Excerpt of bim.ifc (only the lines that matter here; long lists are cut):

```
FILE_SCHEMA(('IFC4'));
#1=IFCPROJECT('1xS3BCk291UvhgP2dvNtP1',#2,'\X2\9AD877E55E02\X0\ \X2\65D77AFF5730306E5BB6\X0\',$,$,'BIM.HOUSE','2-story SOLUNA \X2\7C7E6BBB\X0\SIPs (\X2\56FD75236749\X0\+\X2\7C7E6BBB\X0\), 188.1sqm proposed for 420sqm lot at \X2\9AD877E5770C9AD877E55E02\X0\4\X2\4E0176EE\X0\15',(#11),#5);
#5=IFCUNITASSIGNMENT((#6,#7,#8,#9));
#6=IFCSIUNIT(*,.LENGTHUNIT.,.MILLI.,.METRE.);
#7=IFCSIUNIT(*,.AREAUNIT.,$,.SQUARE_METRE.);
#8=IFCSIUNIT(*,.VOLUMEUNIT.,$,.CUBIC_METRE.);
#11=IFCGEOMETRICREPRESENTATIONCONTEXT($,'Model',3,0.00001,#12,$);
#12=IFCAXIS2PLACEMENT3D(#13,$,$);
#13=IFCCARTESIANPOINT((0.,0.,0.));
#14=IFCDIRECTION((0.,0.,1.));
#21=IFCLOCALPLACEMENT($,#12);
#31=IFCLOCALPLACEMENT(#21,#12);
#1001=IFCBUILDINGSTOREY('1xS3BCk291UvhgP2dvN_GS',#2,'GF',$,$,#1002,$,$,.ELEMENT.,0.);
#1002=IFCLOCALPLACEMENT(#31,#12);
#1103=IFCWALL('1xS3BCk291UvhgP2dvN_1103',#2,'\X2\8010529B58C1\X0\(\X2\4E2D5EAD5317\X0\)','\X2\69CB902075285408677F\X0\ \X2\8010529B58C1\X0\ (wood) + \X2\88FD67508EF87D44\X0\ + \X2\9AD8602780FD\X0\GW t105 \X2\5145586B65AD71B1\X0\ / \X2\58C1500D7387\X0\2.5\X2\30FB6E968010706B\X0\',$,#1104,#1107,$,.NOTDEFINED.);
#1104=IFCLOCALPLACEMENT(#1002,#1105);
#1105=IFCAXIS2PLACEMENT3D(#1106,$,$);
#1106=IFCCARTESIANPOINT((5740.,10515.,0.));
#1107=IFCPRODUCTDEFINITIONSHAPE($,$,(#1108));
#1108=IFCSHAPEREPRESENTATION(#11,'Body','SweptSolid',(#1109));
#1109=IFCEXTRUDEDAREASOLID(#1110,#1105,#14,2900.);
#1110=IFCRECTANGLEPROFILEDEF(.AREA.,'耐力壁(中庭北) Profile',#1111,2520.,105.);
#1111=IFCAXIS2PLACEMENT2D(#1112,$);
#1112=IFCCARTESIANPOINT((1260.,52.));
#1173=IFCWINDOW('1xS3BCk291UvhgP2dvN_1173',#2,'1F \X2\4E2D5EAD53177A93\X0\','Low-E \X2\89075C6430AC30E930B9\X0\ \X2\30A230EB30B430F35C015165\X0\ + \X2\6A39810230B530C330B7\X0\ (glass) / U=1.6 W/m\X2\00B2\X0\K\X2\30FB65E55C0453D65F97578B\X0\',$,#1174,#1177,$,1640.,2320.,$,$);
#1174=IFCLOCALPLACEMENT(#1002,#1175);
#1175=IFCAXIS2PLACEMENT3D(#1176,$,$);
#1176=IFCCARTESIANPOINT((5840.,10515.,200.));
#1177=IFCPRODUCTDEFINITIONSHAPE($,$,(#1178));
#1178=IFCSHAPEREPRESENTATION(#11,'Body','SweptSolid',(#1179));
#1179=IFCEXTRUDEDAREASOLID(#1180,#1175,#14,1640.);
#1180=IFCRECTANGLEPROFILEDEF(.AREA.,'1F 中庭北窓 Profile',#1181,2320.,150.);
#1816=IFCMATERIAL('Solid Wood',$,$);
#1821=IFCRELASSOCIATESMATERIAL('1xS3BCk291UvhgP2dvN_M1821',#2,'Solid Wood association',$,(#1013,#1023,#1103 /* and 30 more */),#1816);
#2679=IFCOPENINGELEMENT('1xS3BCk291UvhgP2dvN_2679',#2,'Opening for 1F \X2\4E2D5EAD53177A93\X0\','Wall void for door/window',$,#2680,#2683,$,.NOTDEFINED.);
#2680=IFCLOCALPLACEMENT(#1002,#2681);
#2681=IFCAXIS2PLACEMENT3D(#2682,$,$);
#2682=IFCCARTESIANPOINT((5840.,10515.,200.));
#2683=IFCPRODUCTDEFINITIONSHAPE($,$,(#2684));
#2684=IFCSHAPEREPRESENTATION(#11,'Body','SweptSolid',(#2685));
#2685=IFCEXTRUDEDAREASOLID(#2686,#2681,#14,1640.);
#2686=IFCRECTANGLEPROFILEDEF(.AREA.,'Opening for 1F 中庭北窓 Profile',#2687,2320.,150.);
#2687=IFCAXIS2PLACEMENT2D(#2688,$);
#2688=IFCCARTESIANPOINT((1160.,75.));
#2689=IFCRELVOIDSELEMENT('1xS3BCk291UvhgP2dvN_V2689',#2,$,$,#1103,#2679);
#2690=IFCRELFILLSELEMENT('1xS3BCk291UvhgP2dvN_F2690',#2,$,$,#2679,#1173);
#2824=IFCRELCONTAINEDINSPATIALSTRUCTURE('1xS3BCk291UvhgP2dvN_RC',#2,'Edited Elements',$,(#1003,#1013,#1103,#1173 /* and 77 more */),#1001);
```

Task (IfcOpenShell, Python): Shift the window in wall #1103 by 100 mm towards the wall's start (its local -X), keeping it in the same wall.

```python
import ifcopenshell
import ifcopenshell.api.geometry
import ifcopenshell.util.placement
import ifcopenshell.util.unit

model = ifcopenshell.open("bim.ifc")
unit_scale = ifcopenshell.util.unit.calculate_unit_scale(model)

window = model.by_id(1173)
opening = window.FillsVoids[0].RelatingOpeningElement
wall = opening.VoidsElements[0].RelatingBuildingElement

wall_matrix = ifcopenshell.util.placement.get_local_placement(wall.ObjectPlacement)
shift = wall_matrix[:3, 0] * -0.1 / unit_scale
before = ifcopenshell.util.placement.get_local_placement(window.ObjectPlacement)[:3, 3].copy()

# The window is not placed relative to its opening, so move both.
for product in (opening, window):
    matrix = ifcopenshell.util.placement.get_local_placement(product.ObjectPlacement)
    matrix[:3, 3] += shift
    ifcopenshell.api.geometry.edit_object_placement(model, product=product, matrix=matrix, is_si=False)

after = ifcopenshell.util.placement.get_local_placement(window.ObjectPlacement)[:3, 3]
print("window moved by", (after - before).round(3) + 0.0)

model.write("bim_updated.ifc")
```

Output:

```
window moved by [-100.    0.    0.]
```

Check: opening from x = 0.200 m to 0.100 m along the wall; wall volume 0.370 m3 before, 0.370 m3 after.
